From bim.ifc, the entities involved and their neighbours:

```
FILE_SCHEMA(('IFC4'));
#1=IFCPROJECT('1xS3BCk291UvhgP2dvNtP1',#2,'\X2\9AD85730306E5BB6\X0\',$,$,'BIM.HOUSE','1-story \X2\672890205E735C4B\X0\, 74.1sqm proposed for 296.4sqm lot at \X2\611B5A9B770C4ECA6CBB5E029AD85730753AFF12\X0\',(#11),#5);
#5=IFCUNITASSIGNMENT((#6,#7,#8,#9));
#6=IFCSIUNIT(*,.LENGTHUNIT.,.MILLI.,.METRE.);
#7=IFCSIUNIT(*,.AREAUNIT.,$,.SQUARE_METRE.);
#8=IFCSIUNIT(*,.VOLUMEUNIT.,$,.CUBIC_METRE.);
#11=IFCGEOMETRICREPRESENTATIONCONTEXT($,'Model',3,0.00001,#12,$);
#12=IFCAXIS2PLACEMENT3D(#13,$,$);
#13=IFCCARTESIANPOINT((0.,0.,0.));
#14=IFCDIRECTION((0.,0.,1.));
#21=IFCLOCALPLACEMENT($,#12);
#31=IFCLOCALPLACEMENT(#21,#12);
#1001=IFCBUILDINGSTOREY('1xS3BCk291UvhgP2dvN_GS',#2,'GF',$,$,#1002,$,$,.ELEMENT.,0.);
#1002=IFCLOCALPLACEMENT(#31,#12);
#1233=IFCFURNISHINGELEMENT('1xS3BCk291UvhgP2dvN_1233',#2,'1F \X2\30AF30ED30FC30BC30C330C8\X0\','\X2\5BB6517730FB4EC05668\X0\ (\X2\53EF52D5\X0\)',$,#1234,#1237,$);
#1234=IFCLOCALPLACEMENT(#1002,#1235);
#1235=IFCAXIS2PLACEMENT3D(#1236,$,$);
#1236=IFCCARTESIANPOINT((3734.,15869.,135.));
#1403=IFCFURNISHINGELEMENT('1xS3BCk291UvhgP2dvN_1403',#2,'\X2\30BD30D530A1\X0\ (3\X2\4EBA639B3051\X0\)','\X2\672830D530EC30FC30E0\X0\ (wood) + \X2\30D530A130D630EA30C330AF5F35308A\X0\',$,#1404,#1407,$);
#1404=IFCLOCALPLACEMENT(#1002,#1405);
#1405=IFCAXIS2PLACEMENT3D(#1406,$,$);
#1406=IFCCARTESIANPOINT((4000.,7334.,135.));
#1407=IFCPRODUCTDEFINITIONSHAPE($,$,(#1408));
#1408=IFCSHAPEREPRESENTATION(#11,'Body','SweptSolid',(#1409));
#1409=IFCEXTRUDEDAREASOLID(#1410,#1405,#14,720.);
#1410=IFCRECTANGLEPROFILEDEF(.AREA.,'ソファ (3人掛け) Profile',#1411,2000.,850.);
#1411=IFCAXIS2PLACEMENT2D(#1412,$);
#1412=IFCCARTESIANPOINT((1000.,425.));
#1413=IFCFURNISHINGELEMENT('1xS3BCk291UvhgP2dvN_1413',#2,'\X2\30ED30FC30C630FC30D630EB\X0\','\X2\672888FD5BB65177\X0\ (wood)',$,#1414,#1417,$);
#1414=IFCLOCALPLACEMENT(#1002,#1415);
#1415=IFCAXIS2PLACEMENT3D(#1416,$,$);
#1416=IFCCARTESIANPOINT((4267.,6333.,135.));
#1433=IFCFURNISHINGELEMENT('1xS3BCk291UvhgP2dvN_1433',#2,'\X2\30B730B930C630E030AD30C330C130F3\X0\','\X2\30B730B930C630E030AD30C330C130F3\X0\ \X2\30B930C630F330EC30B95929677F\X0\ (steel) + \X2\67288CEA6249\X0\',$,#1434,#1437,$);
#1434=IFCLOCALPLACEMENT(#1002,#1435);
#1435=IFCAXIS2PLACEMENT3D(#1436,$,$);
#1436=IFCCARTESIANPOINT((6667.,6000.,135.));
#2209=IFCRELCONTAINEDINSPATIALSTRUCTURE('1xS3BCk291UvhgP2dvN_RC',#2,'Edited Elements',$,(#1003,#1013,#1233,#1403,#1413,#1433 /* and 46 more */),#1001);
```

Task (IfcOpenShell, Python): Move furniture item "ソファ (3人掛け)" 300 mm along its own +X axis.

```python
import ifcopenshell
import ifcopenshell.api.geometry
import ifcopenshell.util.placement
import ifcopenshell.util.unit

model = ifcopenshell.open("bim.ifc")
unit_scale = ifcopenshell.util.unit.calculate_unit_scale(model)

item = model.by_guid("1xS3BCk291UvhgP2dvN_1403")
matrix = ifcopenshell.util.placement.get_local_placement(item.ObjectPlacement)
matrix[:3, 3] += matrix[:3, 0] * 0.3 / unit_scale
ifcopenshell.api.geometry.edit_object_placement(model, product=item, matrix=matrix, is_si=False)

print(ifcopenshell.util.placement.get_local_placement(item.ObjectPlacement).round(3) + 0.0)

model.write("bim-out.ifc")
```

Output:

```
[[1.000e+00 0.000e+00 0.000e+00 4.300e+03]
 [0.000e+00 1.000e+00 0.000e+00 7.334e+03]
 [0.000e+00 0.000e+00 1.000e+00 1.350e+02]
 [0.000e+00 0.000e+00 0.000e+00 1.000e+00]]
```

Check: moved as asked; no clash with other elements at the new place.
